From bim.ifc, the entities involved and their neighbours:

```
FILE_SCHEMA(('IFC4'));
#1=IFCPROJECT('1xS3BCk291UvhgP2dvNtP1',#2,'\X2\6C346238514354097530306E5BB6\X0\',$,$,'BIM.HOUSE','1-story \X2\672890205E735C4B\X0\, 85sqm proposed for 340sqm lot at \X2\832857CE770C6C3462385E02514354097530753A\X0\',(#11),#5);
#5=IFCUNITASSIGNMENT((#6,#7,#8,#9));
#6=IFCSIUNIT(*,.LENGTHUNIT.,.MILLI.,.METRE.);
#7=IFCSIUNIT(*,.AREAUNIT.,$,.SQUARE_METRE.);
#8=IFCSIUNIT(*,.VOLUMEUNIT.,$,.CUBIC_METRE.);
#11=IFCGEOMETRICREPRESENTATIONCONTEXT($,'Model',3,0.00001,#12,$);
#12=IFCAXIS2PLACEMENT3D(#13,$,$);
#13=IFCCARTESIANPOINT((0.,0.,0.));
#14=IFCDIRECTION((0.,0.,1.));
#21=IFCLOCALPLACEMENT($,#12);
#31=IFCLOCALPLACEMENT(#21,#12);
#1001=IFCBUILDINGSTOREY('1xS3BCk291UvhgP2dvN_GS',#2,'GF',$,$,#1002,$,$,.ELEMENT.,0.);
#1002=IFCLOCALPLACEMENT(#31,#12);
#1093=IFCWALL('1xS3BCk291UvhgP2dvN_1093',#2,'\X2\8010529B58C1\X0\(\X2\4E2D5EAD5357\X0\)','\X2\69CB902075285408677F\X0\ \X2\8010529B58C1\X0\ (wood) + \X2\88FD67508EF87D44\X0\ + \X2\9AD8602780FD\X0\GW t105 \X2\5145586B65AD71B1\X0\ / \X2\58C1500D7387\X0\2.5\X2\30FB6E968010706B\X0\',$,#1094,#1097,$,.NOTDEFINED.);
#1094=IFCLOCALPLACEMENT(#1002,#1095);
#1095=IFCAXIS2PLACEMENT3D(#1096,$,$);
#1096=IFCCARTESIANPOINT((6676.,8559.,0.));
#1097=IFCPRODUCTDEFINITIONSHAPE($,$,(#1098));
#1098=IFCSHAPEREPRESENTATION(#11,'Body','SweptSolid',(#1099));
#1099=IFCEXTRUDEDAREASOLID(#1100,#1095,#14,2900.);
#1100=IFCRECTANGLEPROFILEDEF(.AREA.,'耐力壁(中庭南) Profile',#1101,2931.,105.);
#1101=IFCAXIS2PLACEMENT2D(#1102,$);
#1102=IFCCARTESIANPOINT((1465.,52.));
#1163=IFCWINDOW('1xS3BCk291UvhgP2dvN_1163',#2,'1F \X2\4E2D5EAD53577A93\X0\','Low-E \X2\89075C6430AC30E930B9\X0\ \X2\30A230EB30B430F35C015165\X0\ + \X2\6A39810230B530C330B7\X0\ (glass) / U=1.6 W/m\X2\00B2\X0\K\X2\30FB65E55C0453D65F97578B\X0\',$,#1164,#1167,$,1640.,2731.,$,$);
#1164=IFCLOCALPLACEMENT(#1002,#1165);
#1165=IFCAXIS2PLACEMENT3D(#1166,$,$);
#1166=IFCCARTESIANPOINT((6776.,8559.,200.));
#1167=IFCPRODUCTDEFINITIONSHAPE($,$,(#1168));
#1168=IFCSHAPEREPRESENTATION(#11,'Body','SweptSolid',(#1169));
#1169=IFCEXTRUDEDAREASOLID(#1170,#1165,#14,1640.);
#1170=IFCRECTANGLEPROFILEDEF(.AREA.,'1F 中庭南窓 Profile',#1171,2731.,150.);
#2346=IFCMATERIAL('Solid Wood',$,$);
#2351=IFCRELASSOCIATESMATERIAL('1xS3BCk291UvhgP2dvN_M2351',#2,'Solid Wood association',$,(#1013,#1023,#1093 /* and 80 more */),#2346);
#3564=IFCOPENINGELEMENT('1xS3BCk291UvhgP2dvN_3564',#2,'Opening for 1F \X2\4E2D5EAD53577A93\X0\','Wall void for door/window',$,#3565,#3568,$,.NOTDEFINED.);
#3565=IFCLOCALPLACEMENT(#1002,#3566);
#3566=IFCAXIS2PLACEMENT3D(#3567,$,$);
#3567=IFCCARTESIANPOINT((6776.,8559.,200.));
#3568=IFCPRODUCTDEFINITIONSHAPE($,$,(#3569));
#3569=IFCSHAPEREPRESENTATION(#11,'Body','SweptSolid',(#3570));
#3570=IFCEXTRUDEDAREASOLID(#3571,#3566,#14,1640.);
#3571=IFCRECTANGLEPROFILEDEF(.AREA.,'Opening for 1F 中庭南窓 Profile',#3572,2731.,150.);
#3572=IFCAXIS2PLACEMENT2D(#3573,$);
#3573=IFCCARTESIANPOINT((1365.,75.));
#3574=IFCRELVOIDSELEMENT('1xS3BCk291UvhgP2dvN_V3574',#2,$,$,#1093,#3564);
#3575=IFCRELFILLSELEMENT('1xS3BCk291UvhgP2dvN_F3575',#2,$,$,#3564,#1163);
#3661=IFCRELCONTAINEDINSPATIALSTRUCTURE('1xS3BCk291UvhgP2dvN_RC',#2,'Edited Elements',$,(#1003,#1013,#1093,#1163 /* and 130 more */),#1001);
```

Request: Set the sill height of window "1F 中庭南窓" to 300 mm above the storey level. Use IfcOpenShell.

```python
import numpy as np
import ifcopenshell
import ifcopenshell.api.geometry
import ifcopenshell.geom
import ifcopenshell.util.element
import ifcopenshell.util.placement
import ifcopenshell.util.shape
import ifcopenshell.util.unit

model = ifcopenshell.open("bim.ifc")
unit_scale = ifcopenshell.util.unit.calculate_unit_scale(model)

window = model.by_guid("1xS3BCk291UvhgP2dvN_1163")
opening = window.FillsVoids[0].RelatingOpeningElement
storey = ifcopenshell.util.element.get_container(window, ifc_class="IfcBuildingStorey")
level = ifcopenshell.util.placement.get_local_placement(storey.ObjectPlacement)[2, 3]

# The opening's origin need not be at the sill, so measure its lowest point.
shape = ifcopenshell.geom.create_shape(ifcopenshell.geom.settings(), opening)
bottom = ifcopenshell.util.shape.get_shape_bottom_elevation(shape, shape.geometry) / unit_scale
dz = level + 0.3 / unit_scale - bottom

shift = np.array([0.0, 0.0, dz])
# The window is not placed relative to its opening, so move both.
for product in (opening, window):
    matrix = ifcopenshell.util.placement.get_local_placement(product.ObjectPlacement)
    matrix[:3, 3] += shift
    ifcopenshell.api.geometry.edit_object_placement(model, product=product, matrix=matrix, is_si=False)

print(f"moved by {dz * unit_scale:+.3f} m")

model.write("bim-out.ifc")
```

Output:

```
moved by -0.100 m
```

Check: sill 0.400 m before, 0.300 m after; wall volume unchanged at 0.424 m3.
